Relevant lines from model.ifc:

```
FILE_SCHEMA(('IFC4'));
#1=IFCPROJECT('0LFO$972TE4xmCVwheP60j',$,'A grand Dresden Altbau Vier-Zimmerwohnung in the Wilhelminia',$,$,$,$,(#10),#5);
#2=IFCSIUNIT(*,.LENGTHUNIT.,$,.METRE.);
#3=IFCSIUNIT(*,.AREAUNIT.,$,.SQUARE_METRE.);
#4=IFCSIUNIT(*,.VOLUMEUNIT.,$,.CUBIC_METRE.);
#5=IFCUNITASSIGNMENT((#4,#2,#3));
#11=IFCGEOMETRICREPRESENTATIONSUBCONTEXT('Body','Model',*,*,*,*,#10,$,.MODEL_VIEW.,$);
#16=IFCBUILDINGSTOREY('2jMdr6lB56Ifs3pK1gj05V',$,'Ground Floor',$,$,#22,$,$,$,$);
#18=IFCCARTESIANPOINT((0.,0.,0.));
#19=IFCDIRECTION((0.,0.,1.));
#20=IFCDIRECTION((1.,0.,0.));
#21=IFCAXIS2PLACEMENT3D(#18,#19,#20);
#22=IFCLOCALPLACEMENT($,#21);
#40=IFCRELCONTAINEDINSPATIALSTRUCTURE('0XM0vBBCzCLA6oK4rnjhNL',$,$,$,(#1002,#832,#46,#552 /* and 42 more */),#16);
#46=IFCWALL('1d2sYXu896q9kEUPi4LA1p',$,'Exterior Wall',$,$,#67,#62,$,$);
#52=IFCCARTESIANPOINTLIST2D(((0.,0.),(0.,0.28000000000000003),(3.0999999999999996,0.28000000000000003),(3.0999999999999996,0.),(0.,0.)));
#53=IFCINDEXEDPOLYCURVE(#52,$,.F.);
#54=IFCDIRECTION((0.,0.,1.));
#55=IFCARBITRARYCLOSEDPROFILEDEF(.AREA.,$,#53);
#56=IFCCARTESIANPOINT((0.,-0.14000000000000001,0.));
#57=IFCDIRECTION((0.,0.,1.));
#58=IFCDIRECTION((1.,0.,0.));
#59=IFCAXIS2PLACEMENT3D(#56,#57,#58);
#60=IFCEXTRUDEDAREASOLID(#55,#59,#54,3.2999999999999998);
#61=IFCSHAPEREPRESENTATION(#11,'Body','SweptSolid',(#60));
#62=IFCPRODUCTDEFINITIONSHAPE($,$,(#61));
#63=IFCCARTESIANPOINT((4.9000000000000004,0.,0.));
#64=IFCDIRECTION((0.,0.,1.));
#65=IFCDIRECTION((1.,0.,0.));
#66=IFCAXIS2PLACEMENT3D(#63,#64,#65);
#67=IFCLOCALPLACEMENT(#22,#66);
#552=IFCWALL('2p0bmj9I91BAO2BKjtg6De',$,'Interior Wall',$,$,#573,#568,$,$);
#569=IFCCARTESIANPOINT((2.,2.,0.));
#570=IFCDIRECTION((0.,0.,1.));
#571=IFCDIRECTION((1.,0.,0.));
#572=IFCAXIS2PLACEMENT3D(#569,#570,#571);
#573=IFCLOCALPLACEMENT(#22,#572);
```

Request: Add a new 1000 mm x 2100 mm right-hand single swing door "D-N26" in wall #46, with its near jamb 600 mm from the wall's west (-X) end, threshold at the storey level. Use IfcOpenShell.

```python
import numpy as np
import ifcopenshell
import ifcopenshell.api.feature
import ifcopenshell.api.geometry
import ifcopenshell.api.root
import ifcopenshell.api.spatial
import ifcopenshell.geom
import ifcopenshell.util.element
import ifcopenshell.util.placement
import ifcopenshell.util.representation
import ifcopenshell.util.shape
import ifcopenshell.util.unit

model = ifcopenshell.open("model.ifc")
unit_scale = ifcopenshell.util.unit.calculate_unit_scale(model)
settings = ifcopenshell.geom.settings()


def volume(element):
    """Net volume in cubic metres, openings subtracted."""
    shape = ifcopenshell.geom.create_shape(settings, element)
    return ifcopenshell.util.shape.get_volume(shape.geometry)


wall = model.by_guid("1d2sYXu896q9kEUPi4LA1p")
storey = ifcopenshell.util.element.get_container(wall, ifc_class="IfcBuildingStorey")
context = ifcopenshell.util.representation.get_context(model, "Model", "Body", "MODEL_VIEW")
before = volume(wall)

width, height, from_end, sill = 1, 2.1, 0.6, 0.0  # metres

# The wall runs along its own X axis, and the end named is its -X end.
wall_shape = ifcopenshell.geom.create_shape(settings, wall)
x, y, z = ifcopenshell.util.shape.get_vertices(wall_shape.geometry).T
start = x.min() + from_end
face, thickness = float(y.min()), float(y.max() - y.min())
wall_matrix = ifcopenshell.util.placement.get_local_placement(wall.ObjectPlacement)
level = ifcopenshell.util.placement.get_local_placement(storey.ObjectPlacement)[2, 3]


def in_wall(x, y):
    """Placement at x, y metres in the wall's axes, at sill height."""
    matrix = wall_matrix.copy()
    matrix[:, 3] = wall_matrix @ np.array([x / unit_scale, y / unit_scale, 0.0, 1.0])
    matrix[2, 3] = level + sill / unit_scale
    return matrix


# Opening: a box that overshoots both wall faces by 50 mm.
opening = ifcopenshell.api.root.create_entity(model, ifc_class="IfcOpeningElement", predefined_type="OPENING")
box = ifcopenshell.api.geometry.add_wall_representation(
    model, context=context, length=width, height=height, thickness=thickness + 0.1
)
ifcopenshell.api.geometry.assign_representation(model, product=opening, representation=box)
ifcopenshell.api.geometry.edit_object_placement(model, product=opening, matrix=in_wall(start, face - 0.05), is_si=False)
ifcopenshell.api.feature.add_feature(model, feature=opening, element=wall)

door = ifcopenshell.api.root.create_entity(model, ifc_class="IfcDoor", name="D-N26", predefined_type="DOOR")
door.OverallWidth, door.OverallHeight = width / unit_scale, height / unit_scale
door.OperationType = "SINGLE_SWING_RIGHT"
body = ifcopenshell.api.geometry.add_door_representation(
    model,
    context=context,
    overall_width=door.OverallWidth,
    overall_height=door.OverallHeight,
    operation_type="SINGLE_SWING_RIGHT",
    lining_properties={"LiningDepth": thickness / unit_scale, "ThresholdDepth": thickness / unit_scale},
)
ifcopenshell.api.geometry.assign_representation(model, product=door, representation=body)
ifcopenshell.api.spatial.assign_container(model, products=[door], relating_structure=storey)
ifcopenshell.api.feature.add_filling(model, opening=opening, element=door)

# The lining spans the wall, so the door starts at the wall face.
ifcopenshell.api.geometry.edit_object_placement(model, product=door, matrix=in_wall(start, face), is_si=False)

after = volume(wall)

print(f"wall volume {before:.3f} -> {after:.3f} m3")

model.write("model_rev.ifc")
```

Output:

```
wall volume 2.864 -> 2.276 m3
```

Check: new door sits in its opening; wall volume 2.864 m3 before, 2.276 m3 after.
